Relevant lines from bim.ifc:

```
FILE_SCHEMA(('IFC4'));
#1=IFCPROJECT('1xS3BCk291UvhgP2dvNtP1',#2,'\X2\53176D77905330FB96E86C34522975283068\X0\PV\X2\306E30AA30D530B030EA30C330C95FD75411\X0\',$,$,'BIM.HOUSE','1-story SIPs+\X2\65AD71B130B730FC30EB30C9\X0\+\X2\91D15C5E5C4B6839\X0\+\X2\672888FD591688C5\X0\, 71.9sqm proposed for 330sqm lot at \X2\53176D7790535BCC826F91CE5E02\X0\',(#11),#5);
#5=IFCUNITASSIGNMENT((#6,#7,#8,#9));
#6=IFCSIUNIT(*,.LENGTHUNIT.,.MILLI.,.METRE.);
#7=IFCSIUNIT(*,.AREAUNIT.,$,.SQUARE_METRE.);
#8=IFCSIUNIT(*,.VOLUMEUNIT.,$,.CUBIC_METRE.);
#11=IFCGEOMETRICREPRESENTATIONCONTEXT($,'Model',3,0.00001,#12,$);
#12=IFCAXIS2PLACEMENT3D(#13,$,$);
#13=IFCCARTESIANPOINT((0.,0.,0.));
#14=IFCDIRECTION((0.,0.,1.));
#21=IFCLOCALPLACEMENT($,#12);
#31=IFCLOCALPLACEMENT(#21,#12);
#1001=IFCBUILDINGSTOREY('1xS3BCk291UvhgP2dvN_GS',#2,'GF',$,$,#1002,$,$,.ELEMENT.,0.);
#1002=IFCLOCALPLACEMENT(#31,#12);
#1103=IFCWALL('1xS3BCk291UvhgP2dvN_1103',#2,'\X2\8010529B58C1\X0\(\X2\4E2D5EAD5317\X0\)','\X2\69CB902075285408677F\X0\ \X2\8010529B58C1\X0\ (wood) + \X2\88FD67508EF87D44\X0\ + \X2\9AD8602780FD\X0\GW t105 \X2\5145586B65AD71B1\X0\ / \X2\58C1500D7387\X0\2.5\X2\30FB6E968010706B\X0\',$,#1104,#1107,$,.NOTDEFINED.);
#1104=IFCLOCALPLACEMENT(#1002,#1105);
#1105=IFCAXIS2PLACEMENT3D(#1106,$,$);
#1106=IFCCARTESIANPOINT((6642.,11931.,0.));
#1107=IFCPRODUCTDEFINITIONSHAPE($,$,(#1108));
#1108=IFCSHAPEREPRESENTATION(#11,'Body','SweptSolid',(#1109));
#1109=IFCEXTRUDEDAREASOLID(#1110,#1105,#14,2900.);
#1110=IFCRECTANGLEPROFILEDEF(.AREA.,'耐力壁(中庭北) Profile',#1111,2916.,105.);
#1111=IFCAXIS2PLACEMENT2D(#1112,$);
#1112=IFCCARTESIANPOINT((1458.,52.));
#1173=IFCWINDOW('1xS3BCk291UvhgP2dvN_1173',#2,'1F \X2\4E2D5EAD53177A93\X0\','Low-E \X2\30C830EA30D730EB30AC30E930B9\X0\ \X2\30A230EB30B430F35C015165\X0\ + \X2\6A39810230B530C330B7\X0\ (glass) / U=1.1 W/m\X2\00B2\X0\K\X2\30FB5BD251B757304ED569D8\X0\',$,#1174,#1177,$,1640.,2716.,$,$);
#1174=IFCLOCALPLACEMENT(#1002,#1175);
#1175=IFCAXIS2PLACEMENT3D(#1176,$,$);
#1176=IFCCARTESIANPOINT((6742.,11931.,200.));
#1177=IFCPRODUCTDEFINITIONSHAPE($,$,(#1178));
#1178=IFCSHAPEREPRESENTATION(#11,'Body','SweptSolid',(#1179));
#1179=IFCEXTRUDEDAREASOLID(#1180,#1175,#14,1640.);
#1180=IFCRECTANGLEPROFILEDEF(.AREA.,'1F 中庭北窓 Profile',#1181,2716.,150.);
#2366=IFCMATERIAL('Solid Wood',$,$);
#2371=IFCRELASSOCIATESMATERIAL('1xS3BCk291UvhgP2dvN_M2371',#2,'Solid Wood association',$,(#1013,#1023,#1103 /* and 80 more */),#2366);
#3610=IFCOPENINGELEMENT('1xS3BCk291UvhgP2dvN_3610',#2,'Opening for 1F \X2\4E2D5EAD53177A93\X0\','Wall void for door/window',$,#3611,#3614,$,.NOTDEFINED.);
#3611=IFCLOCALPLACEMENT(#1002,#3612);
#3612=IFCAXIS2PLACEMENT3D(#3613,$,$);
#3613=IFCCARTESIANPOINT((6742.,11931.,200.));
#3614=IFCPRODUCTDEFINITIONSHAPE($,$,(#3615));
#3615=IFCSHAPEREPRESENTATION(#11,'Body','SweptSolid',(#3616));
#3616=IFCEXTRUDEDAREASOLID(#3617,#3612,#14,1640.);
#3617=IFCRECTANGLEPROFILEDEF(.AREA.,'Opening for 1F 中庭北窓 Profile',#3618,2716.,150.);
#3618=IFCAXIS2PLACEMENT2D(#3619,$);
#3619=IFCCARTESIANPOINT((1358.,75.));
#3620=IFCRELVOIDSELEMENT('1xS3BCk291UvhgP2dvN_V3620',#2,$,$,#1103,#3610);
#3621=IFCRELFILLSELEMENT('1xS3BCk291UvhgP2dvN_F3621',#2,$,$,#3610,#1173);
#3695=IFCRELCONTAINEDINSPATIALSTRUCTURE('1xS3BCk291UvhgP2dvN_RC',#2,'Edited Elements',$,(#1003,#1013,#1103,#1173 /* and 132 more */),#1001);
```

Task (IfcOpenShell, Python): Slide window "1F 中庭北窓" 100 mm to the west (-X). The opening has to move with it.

```python
import ifcopenshell
import ifcopenshell.api.geometry
import ifcopenshell.util.placement
import ifcopenshell.util.unit

model = ifcopenshell.open("bim.ifc")
unit_scale = ifcopenshell.util.unit.calculate_unit_scale(model)

window = model.by_guid("1xS3BCk291UvhgP2dvN_1173")
opening = window.FillsVoids[0].RelatingOpeningElement
wall = opening.VoidsElements[0].RelatingBuildingElement

wall_matrix = ifcopenshell.util.placement.get_local_placement(wall.ObjectPlacement)
shift = wall_matrix[:3, 0] * -0.1 / unit_scale
before = ifcopenshell.util.placement.get_local_placement(window.ObjectPlacement)[:3, 3].copy()

# The window is not placed relative to its opening, so move both.
for product in (opening, window):
    matrix = ifcopenshell.util.placement.get_local_placement(product.ObjectPlacement)
    matrix[:3, 3] += shift
    ifcopenshell.api.geometry.edit_object_placement(model, product=product, matrix=matrix, is_si=False)

after = ifcopenshell.util.placement.get_local_placement(window.ObjectPlacement)[:3, 3]
print("window moved by", (after - before).round(3) + 0.0)

model.write("bim_edited.ifc")
```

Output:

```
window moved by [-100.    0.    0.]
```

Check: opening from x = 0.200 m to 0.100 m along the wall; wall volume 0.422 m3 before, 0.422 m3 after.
